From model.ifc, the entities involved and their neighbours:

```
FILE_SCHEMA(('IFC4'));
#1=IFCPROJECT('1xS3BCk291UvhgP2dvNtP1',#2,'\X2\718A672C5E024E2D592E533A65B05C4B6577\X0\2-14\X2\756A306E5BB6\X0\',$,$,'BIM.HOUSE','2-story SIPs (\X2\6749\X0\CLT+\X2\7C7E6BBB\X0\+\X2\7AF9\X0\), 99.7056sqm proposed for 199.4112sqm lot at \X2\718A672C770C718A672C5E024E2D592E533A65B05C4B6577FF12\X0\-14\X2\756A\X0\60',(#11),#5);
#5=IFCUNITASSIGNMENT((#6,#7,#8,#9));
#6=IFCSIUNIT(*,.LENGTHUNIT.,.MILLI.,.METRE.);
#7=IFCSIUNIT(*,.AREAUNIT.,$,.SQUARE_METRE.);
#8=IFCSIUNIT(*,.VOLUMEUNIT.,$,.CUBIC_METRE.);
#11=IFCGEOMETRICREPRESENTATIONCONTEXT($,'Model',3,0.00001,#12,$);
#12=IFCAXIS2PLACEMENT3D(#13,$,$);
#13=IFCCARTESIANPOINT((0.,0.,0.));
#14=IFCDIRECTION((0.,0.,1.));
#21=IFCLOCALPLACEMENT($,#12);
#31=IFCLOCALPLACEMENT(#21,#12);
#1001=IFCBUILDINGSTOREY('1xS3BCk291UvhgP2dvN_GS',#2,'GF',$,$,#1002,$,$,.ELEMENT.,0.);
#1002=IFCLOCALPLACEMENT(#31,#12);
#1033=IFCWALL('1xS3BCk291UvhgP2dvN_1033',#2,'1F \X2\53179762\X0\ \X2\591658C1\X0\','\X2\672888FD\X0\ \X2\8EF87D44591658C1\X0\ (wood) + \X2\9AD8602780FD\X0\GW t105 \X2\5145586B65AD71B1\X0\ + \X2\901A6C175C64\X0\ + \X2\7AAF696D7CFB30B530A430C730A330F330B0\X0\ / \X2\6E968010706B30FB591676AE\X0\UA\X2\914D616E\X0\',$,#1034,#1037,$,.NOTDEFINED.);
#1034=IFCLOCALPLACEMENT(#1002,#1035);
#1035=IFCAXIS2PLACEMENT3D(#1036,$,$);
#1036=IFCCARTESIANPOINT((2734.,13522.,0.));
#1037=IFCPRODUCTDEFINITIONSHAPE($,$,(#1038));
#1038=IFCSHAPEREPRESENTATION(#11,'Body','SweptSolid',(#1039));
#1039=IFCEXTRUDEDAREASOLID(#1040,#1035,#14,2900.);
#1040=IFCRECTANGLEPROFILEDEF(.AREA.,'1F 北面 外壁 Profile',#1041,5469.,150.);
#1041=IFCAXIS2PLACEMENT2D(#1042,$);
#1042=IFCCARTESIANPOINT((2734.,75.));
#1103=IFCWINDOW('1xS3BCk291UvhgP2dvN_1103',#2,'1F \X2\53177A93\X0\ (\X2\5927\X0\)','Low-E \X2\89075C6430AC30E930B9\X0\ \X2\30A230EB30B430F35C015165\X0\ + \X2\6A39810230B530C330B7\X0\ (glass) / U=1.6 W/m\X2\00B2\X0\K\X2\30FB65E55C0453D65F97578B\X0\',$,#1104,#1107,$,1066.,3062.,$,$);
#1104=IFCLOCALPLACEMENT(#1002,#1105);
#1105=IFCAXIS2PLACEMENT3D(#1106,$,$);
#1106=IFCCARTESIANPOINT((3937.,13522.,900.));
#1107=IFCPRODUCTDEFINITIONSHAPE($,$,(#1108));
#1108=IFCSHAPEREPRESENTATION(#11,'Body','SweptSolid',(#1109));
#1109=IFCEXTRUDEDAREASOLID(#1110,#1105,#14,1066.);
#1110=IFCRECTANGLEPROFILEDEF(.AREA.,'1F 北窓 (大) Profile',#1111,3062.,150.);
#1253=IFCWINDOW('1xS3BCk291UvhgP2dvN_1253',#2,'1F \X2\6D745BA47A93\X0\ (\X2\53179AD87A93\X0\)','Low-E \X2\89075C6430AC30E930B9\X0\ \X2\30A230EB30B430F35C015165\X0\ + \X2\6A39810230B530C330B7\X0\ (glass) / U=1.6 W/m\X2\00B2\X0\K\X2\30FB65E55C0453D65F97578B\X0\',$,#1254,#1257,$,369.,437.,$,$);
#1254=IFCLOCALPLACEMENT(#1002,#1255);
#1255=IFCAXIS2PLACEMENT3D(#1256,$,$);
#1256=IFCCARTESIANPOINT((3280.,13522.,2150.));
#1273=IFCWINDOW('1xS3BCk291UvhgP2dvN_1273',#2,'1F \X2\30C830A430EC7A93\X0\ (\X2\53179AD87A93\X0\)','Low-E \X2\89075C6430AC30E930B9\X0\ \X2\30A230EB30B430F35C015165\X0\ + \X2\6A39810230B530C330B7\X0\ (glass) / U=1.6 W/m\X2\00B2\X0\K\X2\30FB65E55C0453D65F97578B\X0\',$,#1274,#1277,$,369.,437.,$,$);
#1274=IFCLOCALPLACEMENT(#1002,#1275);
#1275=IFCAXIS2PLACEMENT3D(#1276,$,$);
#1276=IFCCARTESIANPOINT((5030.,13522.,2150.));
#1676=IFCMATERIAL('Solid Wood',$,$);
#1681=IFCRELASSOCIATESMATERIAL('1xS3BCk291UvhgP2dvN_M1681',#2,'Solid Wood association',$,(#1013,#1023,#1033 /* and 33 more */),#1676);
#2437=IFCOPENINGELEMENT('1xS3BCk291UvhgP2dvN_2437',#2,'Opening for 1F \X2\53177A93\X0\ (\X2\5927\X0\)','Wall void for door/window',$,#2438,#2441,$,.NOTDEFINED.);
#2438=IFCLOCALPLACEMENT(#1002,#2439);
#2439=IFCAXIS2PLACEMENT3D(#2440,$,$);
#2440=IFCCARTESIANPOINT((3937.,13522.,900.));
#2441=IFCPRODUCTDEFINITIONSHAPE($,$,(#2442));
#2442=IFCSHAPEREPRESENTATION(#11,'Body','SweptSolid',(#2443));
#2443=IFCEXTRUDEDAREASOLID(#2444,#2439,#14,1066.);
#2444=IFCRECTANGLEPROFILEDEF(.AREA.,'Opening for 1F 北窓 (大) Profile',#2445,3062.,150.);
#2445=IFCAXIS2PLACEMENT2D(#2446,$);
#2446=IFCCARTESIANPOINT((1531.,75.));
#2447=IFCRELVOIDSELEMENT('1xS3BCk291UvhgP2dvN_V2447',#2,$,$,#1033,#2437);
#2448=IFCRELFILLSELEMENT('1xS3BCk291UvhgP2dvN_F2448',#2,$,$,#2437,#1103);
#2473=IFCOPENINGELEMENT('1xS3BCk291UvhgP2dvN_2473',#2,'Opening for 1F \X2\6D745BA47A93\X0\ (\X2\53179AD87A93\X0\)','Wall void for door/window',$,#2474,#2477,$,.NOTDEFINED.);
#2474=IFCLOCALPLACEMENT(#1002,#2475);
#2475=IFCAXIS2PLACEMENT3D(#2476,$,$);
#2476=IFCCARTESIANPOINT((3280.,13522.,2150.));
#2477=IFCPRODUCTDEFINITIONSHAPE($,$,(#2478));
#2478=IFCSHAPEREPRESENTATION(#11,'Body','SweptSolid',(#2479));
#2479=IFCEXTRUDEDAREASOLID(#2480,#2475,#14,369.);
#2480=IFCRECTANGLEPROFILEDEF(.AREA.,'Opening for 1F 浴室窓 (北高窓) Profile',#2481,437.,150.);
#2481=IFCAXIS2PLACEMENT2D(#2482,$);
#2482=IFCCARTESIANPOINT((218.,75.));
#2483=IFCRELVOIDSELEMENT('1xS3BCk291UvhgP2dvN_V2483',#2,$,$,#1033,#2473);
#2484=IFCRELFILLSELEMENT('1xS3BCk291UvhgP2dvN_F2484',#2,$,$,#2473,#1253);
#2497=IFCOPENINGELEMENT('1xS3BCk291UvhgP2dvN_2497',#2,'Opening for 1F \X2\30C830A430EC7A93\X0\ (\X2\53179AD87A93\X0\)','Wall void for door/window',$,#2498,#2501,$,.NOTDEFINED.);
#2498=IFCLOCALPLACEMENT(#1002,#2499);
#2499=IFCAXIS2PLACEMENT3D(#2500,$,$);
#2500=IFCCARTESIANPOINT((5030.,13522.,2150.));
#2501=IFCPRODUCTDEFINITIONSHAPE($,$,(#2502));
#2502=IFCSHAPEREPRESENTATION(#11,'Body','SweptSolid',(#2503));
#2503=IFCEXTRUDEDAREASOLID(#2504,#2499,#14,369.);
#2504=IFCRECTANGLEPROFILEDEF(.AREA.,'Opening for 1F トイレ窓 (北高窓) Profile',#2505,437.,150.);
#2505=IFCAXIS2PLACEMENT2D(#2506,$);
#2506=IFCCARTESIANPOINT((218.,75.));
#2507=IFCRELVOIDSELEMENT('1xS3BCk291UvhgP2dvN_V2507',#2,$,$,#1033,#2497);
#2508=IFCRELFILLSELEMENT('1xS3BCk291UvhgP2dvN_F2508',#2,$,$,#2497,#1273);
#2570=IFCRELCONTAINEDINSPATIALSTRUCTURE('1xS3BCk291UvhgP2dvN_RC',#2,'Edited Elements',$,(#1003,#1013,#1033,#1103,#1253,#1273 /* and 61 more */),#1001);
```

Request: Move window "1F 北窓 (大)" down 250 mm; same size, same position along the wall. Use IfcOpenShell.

```python
import numpy as np
import ifcopenshell
import ifcopenshell.api.geometry
import ifcopenshell.util.placement
import ifcopenshell.util.unit

model = ifcopenshell.open("model.ifc")
unit_scale = ifcopenshell.util.unit.calculate_unit_scale(model)

window = model.by_id(1103)
opening = window.FillsVoids[0].RelatingOpeningElement
dz = -0.25 / unit_scale

shift = np.array([0.0, 0.0, dz])
# The window is not placed relative to its opening, so move both.
for product in (opening, window):
    matrix = ifcopenshell.util.placement.get_local_placement(product.ObjectPlacement)
    matrix[:3, 3] += shift
    ifcopenshell.api.geometry.edit_object_placement(model, product=product, matrix=matrix, is_si=False)

print(f"moved by {dz * unit_scale:+.3f} m")

model.write("model-out.ifc")
```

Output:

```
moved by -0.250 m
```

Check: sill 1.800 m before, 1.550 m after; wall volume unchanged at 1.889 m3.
